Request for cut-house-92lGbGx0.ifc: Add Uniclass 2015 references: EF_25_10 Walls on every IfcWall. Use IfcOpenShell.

First a look at what the model holds.

```python
import ifcopenshell

model = ifcopenshell.open("cut-house-92lGbGx0.ifc")
print(model.schema)
print("classifications:", [c.Name for c in model.by_type("IfcClassification")])
for ifc_class in ("IfcDoor", "IfcRoof", "IfcStair", "IfcWall", "IfcWindow"):
    print(ifc_class, len(model.by_type(ifc_class)))
```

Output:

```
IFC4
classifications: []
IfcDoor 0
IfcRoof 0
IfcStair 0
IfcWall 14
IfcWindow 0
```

```python
import ifcopenshell
import ifcopenshell.api.classification

model = ifcopenshell.open("cut-house-92lGbGx0.ifc")

system = ifcopenshell.api.classification.add_classification(model, classification="Uniclass 2015")

codes = {
    "IfcWall": ("EF_25_10", "Walls"),
}
for ifc_class, (code, name) in codes.items():
    products = model.by_type(ifc_class)
    ifcopenshell.api.classification.add_reference(
        model, products=products, classification=system, identification=code, name=name
    )
    print(code, len(products))

model.write("cut-house-92lGbGx0_edited.ifc")
```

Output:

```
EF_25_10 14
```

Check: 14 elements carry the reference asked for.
